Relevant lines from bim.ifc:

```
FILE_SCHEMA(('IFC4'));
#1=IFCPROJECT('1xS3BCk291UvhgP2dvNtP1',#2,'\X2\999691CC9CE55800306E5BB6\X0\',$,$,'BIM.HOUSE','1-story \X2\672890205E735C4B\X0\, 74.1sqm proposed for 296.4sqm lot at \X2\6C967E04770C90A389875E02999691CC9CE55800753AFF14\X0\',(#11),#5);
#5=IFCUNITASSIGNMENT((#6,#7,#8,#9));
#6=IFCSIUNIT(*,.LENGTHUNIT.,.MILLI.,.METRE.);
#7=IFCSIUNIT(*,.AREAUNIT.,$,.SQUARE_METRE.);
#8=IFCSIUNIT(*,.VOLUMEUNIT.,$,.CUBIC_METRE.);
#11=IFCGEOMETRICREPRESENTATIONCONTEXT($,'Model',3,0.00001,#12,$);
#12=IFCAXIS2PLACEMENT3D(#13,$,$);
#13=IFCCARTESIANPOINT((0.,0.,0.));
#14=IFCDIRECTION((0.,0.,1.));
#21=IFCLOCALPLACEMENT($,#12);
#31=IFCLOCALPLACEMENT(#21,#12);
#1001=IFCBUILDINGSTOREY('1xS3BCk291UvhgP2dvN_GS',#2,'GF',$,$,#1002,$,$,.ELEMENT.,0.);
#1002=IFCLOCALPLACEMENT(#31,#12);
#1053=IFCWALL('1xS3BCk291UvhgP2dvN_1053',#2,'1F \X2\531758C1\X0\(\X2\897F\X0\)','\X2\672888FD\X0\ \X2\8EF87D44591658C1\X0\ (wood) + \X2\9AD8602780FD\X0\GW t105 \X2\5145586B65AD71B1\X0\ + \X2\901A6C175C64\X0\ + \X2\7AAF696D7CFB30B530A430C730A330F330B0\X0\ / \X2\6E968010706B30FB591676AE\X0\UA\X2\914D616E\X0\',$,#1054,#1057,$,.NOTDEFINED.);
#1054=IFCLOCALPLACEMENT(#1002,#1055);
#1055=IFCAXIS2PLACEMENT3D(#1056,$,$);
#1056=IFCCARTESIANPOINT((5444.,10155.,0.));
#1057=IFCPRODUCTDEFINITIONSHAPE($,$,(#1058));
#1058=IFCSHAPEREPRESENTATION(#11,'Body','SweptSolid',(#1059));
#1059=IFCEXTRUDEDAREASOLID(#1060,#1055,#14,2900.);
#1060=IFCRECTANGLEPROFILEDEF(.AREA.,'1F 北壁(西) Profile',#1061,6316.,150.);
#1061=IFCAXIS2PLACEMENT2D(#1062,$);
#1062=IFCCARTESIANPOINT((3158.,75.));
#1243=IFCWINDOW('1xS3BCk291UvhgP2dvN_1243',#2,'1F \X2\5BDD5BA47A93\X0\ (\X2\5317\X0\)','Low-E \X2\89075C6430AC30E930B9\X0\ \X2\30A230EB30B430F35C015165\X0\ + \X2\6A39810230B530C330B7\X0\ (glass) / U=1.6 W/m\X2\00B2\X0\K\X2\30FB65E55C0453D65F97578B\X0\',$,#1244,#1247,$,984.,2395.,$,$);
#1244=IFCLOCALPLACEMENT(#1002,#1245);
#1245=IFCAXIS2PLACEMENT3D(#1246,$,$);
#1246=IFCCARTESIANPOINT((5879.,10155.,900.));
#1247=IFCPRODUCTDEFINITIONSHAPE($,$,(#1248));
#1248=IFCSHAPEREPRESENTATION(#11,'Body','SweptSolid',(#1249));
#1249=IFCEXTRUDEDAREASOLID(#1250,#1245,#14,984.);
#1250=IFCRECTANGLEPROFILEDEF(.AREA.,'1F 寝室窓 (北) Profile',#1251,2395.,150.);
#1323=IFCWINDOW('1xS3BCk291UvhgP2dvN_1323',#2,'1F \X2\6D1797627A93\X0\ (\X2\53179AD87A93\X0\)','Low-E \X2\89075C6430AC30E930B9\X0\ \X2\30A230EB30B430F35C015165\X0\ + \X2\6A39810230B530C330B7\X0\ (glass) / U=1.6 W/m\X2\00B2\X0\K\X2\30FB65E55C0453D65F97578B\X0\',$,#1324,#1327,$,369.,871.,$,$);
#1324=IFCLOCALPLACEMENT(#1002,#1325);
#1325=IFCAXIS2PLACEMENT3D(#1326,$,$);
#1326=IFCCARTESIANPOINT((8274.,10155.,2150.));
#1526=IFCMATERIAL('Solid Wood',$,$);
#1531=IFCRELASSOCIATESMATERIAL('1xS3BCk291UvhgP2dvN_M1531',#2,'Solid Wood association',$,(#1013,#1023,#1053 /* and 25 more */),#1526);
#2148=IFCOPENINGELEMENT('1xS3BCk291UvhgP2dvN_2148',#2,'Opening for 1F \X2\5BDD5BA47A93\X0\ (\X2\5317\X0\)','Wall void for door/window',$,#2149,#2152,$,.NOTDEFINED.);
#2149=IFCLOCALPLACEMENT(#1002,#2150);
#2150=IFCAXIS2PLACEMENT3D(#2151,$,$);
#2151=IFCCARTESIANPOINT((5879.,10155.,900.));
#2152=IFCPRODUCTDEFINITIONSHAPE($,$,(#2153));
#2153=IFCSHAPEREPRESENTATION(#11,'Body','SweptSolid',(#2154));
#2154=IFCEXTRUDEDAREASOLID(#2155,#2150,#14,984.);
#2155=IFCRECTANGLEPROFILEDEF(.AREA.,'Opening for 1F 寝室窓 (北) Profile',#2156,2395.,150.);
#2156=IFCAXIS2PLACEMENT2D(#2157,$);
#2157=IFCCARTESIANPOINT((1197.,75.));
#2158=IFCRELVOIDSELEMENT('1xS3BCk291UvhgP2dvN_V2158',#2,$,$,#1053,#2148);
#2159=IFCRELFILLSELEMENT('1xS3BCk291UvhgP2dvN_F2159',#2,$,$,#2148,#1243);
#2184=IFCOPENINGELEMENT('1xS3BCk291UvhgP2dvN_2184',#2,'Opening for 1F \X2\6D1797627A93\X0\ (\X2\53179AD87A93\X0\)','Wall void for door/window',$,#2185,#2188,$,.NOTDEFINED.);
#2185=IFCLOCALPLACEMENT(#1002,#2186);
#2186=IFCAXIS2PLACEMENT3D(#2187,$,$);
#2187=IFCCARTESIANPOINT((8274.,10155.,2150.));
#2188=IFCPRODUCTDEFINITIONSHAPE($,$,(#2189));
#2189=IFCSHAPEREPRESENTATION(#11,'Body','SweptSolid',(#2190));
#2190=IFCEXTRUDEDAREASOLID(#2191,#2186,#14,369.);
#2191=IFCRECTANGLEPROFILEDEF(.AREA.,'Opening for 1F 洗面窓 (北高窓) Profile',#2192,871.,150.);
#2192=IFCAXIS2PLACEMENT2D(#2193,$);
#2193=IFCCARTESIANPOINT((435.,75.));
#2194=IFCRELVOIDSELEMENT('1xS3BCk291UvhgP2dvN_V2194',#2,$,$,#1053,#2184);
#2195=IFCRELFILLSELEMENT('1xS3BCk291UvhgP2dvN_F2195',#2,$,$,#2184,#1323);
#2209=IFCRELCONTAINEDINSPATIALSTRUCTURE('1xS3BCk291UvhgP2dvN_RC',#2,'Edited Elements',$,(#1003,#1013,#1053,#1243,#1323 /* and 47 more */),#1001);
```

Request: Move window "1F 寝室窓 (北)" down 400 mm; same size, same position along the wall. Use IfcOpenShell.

```python
import numpy as np
import ifcopenshell
import ifcopenshell.api.geometry
import ifcopenshell.util.placement
import ifcopenshell.util.unit

model = ifcopenshell.open("bim.ifc")
unit_scale = ifcopenshell.util.unit.calculate_unit_scale(model)

window = model.by_guid("1xS3BCk291UvhgP2dvN_1243")
opening = window.FillsVoids[0].RelatingOpeningElement
dz = -400.0

shift = np.array([0.0, 0.0, dz])
# The window is not placed relative to its opening, so move both.
for product in (opening, window):
    matrix = ifcopenshell.util.placement.get_local_placement(product.ObjectPlacement)
    matrix[:3, 3] += shift
    ifcopenshell.api.geometry.edit_object_placement(model, product=product, matrix=matrix, is_si=False)

print(f"moved by {dz * unit_scale:+.3f} m")

model.write("bim-out.ifc")
```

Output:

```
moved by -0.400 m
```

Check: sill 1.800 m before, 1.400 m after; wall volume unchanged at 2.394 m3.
